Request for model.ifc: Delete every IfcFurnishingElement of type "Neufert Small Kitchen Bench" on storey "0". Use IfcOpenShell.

First a look at what the model holds.

```python
import ifcopenshell
import ifcopenshell.util.element

model = ifcopenshell.open("model.ifc")
print(model.schema)
storey = next(s for s in model.by_type("IfcBuildingStorey") if s.Name == "0")
furniture = [e for e in ifcopenshell.util.element.get_decomposition(storey) if e.is_a("IfcFurnishingElement")]
seen = {}
for e in furniture:
    element_type = ifcopenshell.util.element.get_type(e)
    name = element_type.Name if element_type not in (None, e) else None
    seen[name] = seen.get(name, 0) + 1
for name, count in sorted(seen.items(), key=str):
    print(count, "x", name)
```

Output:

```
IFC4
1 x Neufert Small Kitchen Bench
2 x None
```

```python
import ifcopenshell
import ifcopenshell.api.root
import ifcopenshell.util.element

model = ifcopenshell.open("model.ifc")

storey = next(s for s in model.by_type("IfcBuildingStorey") if s.Name == "0")
furniture = [e for e in ifcopenshell.util.element.get_decomposition(storey) if e.is_a("IfcFurnishingElement")]
targets = [e for e in furniture if (t := ifcopenshell.util.element.get_type(e)) not in (None, e) and t.Name == "Neufert Small Kitchen Bench"]

for e in targets:
    ifcopenshell.api.root.remove_product(model, product=e)
print(len(targets), "removed")

model.write("model_updated.ifc")
```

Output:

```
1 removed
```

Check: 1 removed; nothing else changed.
